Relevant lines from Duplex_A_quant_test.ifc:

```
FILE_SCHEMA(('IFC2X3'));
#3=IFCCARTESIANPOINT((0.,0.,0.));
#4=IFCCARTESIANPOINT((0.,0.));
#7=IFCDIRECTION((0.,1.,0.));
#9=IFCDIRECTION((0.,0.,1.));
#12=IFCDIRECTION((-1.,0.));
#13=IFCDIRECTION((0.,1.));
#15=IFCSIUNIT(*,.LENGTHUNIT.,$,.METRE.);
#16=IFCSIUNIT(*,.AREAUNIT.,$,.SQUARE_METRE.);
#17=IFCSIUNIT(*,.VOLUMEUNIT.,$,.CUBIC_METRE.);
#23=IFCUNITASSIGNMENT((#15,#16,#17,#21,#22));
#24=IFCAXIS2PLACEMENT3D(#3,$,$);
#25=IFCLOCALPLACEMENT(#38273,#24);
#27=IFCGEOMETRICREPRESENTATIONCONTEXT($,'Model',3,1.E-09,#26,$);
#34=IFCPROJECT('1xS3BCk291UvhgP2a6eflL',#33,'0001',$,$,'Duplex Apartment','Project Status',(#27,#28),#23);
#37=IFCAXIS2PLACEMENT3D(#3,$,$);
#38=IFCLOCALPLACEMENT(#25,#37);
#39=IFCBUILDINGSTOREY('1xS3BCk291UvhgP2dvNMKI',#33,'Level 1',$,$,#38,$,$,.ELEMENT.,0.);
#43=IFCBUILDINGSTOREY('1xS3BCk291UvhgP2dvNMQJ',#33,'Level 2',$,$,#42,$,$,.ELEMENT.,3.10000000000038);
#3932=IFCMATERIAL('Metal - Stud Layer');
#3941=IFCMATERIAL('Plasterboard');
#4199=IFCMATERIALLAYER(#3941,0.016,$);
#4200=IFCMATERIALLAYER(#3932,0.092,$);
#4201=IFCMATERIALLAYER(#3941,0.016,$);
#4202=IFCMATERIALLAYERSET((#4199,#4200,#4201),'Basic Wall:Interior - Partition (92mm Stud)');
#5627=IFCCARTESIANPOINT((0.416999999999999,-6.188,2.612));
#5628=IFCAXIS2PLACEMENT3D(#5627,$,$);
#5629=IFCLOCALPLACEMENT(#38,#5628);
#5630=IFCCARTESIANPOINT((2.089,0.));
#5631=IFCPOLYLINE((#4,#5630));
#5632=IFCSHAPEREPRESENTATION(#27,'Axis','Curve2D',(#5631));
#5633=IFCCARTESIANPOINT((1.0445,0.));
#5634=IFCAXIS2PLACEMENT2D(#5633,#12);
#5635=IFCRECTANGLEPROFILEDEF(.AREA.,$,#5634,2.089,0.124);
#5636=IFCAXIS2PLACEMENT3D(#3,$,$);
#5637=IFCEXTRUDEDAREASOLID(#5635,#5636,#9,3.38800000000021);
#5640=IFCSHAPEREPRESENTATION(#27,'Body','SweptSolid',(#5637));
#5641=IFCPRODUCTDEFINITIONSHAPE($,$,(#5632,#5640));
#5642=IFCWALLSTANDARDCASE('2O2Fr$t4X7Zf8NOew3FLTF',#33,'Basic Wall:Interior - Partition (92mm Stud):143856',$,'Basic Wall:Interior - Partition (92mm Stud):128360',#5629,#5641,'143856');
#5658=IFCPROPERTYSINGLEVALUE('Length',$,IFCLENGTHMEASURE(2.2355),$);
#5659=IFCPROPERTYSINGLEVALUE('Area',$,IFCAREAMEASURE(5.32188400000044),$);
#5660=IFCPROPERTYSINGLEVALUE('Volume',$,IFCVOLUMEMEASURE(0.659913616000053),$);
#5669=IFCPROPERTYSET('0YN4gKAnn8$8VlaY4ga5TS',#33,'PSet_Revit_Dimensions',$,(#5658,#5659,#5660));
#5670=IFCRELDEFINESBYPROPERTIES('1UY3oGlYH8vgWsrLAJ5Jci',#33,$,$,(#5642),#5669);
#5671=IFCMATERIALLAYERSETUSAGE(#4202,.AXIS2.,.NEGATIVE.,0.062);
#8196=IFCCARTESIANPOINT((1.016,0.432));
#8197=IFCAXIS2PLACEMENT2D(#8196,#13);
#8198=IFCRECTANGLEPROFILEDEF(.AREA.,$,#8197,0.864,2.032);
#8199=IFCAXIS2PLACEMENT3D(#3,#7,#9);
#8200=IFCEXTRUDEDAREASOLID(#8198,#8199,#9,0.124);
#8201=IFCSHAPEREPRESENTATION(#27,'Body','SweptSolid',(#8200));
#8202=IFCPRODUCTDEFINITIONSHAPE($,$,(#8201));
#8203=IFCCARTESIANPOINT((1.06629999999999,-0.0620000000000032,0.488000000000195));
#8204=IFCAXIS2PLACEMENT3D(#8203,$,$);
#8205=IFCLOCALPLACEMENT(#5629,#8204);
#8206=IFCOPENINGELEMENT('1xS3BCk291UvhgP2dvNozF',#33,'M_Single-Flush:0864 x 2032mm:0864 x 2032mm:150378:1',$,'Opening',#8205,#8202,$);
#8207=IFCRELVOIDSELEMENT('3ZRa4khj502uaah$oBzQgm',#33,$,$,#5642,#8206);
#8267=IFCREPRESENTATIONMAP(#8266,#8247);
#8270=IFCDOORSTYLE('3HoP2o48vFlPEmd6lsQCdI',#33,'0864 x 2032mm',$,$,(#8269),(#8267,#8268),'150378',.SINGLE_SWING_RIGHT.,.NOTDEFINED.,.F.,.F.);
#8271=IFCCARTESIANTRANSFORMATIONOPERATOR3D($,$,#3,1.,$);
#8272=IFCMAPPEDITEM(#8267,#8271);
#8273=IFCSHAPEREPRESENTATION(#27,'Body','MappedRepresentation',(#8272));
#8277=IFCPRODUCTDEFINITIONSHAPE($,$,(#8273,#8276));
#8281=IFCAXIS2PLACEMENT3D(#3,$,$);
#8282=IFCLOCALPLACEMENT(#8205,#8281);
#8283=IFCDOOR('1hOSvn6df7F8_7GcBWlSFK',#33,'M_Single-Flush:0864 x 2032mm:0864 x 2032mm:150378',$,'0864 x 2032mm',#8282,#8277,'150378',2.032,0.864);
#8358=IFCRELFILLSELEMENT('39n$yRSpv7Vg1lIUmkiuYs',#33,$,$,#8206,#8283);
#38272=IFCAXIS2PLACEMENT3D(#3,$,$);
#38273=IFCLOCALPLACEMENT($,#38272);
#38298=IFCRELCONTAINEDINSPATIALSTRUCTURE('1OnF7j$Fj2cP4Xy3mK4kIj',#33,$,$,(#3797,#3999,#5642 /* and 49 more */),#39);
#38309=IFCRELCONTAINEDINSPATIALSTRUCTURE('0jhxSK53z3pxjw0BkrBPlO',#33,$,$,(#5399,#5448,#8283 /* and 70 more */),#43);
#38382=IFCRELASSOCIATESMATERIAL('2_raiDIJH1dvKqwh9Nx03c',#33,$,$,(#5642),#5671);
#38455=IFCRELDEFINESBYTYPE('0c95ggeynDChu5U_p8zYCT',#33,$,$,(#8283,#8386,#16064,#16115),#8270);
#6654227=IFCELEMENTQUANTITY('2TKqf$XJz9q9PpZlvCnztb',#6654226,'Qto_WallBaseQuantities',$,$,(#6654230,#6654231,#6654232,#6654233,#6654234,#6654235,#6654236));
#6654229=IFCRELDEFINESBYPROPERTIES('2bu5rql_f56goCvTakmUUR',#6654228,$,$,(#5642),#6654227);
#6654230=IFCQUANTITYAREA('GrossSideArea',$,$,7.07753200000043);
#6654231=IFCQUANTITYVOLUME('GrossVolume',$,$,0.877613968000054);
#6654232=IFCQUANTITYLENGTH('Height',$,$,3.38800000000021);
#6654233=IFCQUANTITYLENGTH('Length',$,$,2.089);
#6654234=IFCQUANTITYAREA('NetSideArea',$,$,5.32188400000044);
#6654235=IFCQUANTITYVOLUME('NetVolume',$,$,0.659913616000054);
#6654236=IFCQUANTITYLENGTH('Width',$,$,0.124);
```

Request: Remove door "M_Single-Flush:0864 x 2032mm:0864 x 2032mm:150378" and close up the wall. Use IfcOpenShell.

```python
import ifcopenshell
import ifcopenshell.api.feature
import ifcopenshell.api.pset
import ifcopenshell.api.root
import ifcopenshell.geom
import ifcopenshell.util.element
import ifcopenshell.util.shape
import ifcopenshell.util.unit

model = ifcopenshell.open("Duplex_A_quant_test.ifc")
area_scale = ifcopenshell.util.unit.calculate_unit_scale(model, "AREAUNIT")
volume_scale = ifcopenshell.util.unit.calculate_unit_scale(model, "VOLUMEUNIT")
settings = ifcopenshell.geom.settings()


def volume(element):
    """Net volume in cubic metres, openings subtracted."""
    shape = ifcopenshell.geom.create_shape(settings, element)
    return ifcopenshell.util.shape.get_volume(shape.geometry)


door = model.by_guid("1hOSvn6df7F8_7GcBWlSFK")
opening = door.FillsVoids[0].RelatingOpeningElement
wall = opening.VoidsElements[0].RelatingBuildingElement
before = volume(wall)

ifcopenshell.api.root.remove_product(model, product=door)
ifcopenshell.api.feature.remove_feature(model, feature=opening)

after = volume(wall)
thickness = 0.124  # wall thickness in metres

# Update the wall's stored quantities.
pset = model.by_id(ifcopenshell.util.element.get_pset(wall, "PSet_Revit_Dimensions", should_inherit=False)["id"])
ifcopenshell.api.pset.edit_pset(model, pset=pset, properties={
    "Area": model.create_entity("IfcAreaMeasure", after / thickness / area_scale),
    "Volume": model.create_entity("IfcVolumeMeasure", after / volume_scale),
})
qto = model.by_id(ifcopenshell.util.element.get_pset(wall, "Qto_WallBaseQuantities", should_inherit=False)["id"])
ifcopenshell.api.pset.edit_qto(model, qto=qto, properties={
    "NetSideArea": after / thickness / area_scale,
    "NetVolume": after / volume_scale,
})

print(f"wall volume {before:.3f} -> {after:.3f} m3")

model.write("Duplex_A_quant_test_updated.ifc")
```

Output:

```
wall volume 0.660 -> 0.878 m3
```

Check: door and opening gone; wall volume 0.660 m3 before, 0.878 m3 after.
